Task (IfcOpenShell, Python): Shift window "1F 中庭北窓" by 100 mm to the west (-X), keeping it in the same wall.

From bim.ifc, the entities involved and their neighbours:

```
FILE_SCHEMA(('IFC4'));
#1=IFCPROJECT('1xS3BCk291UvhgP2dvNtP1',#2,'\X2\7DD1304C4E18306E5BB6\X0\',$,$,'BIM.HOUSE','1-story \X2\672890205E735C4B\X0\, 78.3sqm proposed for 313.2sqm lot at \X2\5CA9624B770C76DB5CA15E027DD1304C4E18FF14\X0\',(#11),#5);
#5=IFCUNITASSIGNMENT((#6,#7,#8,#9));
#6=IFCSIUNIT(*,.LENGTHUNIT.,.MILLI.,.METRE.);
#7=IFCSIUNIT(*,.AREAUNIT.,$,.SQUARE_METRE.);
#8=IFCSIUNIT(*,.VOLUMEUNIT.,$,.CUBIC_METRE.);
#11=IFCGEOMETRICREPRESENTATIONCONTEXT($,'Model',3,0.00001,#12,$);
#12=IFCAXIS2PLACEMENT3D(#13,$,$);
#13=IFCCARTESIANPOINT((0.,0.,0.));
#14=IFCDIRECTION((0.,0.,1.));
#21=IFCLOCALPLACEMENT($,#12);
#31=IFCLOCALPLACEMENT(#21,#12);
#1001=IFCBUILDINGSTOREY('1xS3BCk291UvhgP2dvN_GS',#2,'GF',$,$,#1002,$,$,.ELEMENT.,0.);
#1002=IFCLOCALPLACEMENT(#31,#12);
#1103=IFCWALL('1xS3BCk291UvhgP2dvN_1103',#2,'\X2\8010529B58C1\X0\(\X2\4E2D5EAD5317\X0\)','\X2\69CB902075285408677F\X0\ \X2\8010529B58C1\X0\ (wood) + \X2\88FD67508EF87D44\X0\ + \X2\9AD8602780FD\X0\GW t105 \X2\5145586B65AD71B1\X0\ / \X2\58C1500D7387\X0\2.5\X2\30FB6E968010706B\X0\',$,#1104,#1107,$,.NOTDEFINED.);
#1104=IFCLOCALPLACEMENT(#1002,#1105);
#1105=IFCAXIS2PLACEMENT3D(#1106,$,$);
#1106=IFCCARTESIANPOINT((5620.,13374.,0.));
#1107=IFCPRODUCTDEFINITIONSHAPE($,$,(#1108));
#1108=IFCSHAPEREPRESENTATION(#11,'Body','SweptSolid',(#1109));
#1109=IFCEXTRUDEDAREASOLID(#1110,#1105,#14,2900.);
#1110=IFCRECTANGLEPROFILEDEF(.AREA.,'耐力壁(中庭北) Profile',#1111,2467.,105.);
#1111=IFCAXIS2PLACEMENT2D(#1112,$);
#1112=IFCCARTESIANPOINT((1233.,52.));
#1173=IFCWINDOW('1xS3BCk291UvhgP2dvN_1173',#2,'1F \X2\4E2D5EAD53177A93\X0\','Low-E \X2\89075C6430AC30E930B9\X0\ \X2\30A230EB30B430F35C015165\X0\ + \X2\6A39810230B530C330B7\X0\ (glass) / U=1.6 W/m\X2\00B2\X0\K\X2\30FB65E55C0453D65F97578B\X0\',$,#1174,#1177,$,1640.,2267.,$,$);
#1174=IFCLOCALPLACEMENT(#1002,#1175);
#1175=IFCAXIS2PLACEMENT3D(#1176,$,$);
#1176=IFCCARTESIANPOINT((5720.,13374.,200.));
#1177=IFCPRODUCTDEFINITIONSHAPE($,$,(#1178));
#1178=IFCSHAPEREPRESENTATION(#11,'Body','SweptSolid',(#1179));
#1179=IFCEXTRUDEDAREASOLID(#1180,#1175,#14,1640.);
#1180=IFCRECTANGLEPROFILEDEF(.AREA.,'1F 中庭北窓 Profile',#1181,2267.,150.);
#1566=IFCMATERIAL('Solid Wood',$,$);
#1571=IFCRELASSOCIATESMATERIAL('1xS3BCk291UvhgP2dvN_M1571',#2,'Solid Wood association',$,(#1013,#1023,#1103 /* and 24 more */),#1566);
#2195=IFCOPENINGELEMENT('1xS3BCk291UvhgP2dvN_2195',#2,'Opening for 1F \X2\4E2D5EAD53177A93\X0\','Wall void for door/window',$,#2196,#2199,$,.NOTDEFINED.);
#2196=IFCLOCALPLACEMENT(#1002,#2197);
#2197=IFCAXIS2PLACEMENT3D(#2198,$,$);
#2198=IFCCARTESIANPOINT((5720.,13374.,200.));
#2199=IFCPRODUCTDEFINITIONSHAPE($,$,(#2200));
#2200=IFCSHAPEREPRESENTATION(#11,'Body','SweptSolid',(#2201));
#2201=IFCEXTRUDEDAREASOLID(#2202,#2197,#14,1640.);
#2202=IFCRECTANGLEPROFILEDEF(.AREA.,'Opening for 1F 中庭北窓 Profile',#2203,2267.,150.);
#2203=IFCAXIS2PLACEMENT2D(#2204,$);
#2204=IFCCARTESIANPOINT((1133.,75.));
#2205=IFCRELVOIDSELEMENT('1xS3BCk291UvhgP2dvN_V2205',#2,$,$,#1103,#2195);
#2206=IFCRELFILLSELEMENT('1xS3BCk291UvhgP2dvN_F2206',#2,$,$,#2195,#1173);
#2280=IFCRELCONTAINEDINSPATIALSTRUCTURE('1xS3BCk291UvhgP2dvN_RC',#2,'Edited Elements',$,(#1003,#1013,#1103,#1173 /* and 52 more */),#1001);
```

```python
import ifcopenshell
import ifcopenshell.api.geometry
import ifcopenshell.util.placement

model = ifcopenshell.open("bim.ifc")

window = model.by_id(1173)
opening = window.FillsVoids[0].RelatingOpeningElement
wall = opening.VoidsElements[0].RelatingBuildingElement

wall_matrix = ifcopenshell.util.placement.get_local_placement(wall.ObjectPlacement)
shift = wall_matrix[:3, 0] * -100.0
before = ifcopenshell.util.placement.get_local_placement(window.ObjectPlacement)[:3, 3].copy()

# The window is not placed relative to its opening, so move both.
for product in (opening, window):
    matrix = ifcopenshell.util.placement.get_local_placement(product.ObjectPlacement)
    matrix[:3, 3] += shift
    ifcopenshell.api.geometry.edit_object_placement(model, product=product, matrix=matrix, is_si=False)

after = ifcopenshell.util.placement.get_local_placement(window.ObjectPlacement)[:3, 3]
print("window moved by", (after - before).round(3) + 0.0)

model.write("bim_updated.ifc")
```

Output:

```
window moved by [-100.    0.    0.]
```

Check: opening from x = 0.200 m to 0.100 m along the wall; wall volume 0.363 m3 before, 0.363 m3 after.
